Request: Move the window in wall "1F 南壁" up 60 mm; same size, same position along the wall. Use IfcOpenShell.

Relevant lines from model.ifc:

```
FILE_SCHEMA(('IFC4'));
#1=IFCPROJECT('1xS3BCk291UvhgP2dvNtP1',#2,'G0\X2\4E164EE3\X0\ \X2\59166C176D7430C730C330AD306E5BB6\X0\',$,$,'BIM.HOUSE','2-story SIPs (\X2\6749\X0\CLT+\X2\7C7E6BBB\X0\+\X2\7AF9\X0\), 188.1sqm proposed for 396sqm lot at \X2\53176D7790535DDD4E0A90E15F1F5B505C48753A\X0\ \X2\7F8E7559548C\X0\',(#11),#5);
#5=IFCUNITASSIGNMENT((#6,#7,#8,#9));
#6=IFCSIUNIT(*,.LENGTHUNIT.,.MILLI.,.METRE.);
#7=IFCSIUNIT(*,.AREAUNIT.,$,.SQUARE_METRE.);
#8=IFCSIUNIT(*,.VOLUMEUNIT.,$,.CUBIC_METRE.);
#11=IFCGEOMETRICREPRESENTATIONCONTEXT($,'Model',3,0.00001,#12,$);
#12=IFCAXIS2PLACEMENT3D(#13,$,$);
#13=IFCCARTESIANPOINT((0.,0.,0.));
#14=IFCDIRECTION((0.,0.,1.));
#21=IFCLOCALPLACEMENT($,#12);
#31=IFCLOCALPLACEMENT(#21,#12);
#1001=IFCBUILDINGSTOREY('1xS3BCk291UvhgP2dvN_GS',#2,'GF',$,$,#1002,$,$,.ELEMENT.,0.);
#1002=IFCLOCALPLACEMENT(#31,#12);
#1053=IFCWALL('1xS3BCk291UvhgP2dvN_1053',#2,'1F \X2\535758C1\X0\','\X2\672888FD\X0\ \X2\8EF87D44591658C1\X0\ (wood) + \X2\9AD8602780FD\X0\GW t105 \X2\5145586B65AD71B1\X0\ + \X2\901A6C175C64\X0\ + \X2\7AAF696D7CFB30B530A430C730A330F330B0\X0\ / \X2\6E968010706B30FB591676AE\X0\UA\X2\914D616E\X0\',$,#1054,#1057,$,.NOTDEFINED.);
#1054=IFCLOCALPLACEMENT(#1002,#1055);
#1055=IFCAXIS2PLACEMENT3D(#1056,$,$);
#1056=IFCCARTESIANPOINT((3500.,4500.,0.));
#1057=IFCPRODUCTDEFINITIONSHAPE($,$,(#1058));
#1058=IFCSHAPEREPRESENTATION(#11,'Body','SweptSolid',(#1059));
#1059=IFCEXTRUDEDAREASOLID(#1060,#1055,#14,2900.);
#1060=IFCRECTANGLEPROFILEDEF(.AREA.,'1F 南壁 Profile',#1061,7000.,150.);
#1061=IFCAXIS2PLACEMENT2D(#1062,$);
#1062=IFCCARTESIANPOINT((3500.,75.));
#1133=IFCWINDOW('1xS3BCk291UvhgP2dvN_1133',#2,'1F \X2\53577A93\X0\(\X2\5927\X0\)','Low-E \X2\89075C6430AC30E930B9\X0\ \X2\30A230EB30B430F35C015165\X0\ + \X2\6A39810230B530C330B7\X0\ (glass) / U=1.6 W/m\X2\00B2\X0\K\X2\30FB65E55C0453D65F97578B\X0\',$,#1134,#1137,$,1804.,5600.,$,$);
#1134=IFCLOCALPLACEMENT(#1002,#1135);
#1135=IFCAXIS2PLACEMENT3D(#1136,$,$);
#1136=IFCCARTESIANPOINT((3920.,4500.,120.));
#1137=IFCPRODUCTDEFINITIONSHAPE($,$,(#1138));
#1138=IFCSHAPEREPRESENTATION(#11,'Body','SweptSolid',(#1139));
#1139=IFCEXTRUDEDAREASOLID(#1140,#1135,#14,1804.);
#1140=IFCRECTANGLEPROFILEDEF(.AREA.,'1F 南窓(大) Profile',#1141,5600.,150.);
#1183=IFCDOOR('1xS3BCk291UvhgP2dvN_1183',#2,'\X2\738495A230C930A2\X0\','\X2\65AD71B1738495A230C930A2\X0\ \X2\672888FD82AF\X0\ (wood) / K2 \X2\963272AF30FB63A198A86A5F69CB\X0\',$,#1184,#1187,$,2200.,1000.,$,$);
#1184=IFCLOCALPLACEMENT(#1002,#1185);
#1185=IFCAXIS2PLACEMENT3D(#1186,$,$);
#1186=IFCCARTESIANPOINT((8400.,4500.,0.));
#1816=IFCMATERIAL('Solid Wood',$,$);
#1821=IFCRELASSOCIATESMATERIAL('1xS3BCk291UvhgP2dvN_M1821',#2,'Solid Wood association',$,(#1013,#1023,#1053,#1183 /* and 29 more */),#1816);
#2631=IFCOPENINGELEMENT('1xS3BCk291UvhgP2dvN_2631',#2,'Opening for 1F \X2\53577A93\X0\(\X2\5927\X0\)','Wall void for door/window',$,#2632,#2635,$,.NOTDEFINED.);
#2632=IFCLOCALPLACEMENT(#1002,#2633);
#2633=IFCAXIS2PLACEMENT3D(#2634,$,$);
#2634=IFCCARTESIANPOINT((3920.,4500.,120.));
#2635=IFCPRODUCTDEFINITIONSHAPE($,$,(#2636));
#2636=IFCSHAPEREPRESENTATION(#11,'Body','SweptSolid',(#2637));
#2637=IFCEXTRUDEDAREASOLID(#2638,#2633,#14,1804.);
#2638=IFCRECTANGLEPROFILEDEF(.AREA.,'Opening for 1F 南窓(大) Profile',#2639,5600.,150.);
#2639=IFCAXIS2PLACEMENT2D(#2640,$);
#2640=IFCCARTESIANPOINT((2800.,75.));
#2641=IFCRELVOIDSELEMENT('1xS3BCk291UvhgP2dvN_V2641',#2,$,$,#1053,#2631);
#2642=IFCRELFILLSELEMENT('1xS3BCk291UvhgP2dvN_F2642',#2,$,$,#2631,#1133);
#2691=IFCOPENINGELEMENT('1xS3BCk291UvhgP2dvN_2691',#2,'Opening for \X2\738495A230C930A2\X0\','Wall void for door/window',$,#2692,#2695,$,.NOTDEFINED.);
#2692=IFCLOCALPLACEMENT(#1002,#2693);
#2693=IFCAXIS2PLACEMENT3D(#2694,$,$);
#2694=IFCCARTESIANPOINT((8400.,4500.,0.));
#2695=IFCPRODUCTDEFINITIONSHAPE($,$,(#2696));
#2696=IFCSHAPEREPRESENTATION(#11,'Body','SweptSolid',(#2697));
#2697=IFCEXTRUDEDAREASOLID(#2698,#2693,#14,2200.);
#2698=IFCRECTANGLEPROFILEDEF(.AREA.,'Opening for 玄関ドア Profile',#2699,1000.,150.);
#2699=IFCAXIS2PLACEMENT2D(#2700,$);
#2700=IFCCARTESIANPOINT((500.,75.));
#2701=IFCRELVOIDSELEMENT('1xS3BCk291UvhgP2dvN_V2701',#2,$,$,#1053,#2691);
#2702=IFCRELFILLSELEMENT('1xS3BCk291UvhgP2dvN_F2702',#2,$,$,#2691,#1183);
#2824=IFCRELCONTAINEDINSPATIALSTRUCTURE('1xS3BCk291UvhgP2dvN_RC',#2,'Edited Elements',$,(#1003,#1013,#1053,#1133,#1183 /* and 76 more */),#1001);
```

```python
import numpy as np
import ifcopenshell
import ifcopenshell.api.geometry
import ifcopenshell.util.placement
import ifcopenshell.util.unit

model = ifcopenshell.open("model.ifc")
unit_scale = ifcopenshell.util.unit.calculate_unit_scale(model)

window = model.by_id(1133)
opening = window.FillsVoids[0].RelatingOpeningElement
dz = 60.0

shift = np.array([0.0, 0.0, dz])
# The window is not placed relative to its opening, so move both.
for product in (opening, window):
    matrix = ifcopenshell.util.placement.get_local_placement(product.ObjectPlacement)
    matrix[:3, 3] += shift
    ifcopenshell.api.geometry.edit_object_placement(model, product=product, matrix=matrix, is_si=False)

print(f"moved by {dz * unit_scale:+.3f} m")

model.write("model_rev.ifc")
```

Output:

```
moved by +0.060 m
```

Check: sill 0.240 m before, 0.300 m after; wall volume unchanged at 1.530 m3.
